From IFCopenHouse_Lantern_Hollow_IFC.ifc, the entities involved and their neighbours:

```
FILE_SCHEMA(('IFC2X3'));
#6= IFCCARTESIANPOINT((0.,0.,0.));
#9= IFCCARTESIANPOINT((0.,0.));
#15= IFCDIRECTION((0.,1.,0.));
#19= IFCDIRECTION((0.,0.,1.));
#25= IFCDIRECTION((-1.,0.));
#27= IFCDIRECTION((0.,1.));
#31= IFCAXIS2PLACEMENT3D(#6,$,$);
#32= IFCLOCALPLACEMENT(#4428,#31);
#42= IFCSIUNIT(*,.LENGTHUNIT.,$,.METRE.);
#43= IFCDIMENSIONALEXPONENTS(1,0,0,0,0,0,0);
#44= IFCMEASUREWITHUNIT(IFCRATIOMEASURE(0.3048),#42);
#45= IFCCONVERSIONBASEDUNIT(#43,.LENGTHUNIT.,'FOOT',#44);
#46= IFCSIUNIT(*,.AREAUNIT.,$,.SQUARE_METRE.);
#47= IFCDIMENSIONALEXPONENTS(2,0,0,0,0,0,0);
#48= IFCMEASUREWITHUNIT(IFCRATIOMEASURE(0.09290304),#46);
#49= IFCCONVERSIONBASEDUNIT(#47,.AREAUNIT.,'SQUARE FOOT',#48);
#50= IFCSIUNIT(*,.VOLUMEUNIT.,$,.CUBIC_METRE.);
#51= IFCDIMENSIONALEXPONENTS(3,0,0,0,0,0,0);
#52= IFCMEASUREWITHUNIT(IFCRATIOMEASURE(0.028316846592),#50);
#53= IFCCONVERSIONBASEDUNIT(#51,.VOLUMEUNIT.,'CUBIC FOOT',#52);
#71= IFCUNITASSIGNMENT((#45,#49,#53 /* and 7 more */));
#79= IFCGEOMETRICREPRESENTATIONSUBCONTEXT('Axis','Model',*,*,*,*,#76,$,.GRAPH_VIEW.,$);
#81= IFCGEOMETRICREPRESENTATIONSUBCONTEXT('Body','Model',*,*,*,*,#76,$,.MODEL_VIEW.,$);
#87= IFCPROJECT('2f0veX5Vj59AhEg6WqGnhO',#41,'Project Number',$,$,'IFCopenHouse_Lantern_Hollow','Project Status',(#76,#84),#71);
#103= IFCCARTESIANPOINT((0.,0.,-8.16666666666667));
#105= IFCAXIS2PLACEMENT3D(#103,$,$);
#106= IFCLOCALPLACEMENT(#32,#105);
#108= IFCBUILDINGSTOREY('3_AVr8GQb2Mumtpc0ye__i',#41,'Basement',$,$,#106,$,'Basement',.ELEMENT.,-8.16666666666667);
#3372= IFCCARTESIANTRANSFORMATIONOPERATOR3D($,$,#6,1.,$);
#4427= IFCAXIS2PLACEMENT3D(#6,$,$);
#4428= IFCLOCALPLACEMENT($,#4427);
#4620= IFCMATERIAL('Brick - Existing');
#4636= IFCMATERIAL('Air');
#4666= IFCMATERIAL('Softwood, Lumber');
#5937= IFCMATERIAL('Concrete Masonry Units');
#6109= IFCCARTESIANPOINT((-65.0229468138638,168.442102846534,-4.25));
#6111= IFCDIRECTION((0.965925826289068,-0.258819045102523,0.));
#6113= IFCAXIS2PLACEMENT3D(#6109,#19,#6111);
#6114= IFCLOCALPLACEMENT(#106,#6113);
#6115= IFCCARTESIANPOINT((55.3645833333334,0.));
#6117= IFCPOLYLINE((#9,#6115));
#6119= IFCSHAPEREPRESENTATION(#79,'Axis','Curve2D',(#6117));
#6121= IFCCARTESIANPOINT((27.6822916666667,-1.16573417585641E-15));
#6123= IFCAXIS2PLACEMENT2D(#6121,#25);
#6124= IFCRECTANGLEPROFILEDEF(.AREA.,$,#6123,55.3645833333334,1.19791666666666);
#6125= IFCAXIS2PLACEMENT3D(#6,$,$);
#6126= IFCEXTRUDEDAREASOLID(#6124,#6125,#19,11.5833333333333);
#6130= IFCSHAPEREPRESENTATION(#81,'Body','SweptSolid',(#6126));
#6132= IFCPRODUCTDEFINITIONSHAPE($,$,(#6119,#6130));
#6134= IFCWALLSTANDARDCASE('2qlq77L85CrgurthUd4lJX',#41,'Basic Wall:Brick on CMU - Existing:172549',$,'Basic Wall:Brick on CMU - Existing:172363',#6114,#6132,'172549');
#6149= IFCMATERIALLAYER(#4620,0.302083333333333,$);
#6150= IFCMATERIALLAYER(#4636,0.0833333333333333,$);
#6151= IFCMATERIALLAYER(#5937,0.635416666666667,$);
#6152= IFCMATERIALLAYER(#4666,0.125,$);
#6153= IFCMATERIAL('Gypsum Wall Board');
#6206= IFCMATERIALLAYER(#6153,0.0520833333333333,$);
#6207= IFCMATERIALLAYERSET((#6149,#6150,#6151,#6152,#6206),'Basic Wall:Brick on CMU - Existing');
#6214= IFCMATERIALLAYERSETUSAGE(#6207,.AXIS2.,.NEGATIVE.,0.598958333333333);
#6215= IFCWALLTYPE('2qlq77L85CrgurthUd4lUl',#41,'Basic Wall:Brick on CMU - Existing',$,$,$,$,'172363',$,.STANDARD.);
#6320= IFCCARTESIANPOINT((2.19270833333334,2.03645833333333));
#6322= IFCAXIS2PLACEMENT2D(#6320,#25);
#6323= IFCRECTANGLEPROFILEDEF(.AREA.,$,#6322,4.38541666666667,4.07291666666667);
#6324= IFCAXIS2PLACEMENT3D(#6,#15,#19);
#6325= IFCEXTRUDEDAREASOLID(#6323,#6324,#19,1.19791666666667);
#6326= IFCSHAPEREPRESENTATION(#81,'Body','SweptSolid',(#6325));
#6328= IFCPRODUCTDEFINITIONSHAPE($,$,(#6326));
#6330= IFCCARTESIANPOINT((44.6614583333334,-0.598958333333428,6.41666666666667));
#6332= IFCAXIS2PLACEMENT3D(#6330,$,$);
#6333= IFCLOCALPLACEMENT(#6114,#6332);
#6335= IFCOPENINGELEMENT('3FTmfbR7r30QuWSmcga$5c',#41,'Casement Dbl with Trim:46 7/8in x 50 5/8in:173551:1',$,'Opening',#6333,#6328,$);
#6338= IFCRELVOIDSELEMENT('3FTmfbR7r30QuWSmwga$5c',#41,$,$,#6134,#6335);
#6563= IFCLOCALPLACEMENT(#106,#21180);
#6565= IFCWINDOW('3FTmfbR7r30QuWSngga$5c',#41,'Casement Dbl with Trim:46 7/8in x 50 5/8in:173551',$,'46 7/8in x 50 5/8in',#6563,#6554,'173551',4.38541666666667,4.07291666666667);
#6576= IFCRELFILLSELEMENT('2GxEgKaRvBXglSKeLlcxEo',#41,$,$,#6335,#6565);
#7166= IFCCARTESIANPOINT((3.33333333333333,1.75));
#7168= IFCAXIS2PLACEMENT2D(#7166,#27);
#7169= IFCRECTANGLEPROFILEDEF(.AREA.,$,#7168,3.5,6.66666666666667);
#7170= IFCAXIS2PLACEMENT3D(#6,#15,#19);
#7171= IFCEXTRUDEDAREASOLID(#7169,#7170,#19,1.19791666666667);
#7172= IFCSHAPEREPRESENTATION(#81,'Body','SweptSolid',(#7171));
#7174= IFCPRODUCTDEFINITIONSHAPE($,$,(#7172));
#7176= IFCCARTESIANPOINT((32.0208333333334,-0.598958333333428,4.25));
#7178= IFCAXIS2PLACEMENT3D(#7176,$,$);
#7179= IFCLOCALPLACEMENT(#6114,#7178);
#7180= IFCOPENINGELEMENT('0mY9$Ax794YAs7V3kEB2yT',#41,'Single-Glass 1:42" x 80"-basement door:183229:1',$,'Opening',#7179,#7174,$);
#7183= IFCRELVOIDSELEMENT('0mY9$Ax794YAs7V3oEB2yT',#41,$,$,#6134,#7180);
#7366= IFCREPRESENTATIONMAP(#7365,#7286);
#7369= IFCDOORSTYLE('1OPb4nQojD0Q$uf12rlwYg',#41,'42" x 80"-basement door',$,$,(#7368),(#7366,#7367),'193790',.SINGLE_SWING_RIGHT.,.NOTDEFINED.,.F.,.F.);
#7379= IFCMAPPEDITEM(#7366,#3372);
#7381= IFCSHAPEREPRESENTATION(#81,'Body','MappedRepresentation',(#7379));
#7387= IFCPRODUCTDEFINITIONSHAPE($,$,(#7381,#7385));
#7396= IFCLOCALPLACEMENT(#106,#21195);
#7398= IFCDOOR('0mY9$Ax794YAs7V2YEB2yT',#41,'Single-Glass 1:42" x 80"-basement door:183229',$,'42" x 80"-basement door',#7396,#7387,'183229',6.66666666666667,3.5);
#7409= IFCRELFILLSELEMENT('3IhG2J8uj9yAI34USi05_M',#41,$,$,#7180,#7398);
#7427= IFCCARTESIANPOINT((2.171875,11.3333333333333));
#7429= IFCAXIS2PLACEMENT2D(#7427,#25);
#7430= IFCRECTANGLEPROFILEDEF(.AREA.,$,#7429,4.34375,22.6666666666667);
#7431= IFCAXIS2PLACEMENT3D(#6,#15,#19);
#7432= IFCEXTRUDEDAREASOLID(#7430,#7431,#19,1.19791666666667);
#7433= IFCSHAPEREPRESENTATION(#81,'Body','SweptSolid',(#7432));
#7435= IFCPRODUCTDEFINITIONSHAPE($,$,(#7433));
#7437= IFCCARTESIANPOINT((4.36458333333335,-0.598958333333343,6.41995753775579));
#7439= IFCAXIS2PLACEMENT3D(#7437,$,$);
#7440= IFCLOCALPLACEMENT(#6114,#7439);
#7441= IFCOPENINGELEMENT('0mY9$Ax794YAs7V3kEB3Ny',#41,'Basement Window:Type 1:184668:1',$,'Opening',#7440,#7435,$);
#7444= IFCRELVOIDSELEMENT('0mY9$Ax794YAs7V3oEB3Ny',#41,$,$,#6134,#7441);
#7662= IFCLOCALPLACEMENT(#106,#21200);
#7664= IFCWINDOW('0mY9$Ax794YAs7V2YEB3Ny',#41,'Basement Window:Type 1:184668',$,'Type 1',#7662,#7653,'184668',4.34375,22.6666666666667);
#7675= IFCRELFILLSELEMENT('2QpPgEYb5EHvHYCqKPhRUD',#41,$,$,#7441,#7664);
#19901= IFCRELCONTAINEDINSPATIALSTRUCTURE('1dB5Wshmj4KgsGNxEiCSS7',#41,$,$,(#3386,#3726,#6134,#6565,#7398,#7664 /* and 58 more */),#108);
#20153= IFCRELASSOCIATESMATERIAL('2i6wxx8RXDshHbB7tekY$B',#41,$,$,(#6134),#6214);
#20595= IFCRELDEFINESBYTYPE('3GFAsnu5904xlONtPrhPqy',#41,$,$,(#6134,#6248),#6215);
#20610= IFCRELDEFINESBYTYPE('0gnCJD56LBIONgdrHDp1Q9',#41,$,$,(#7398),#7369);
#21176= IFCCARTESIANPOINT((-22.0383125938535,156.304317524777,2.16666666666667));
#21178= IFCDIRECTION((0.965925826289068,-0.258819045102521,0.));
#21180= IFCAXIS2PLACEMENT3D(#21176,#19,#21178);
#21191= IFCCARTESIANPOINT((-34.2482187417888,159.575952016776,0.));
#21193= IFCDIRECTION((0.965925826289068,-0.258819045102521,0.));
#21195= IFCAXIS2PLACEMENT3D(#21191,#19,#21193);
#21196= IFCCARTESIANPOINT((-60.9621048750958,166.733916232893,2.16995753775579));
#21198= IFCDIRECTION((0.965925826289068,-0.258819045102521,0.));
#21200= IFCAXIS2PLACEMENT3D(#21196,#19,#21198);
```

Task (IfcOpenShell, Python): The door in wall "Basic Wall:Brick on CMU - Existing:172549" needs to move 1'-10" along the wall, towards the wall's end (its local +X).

```python
import ifcopenshell
import ifcopenshell.api.geometry
import ifcopenshell.util.placement
import ifcopenshell.util.unit

model = ifcopenshell.open("IFCopenHouse_Lantern_Hollow_IFC.ifc")
unit_scale = ifcopenshell.util.unit.calculate_unit_scale(model)

door = model.by_guid("0mY9$Ax794YAs7V2YEB2yT")
opening = door.FillsVoids[0].RelatingOpeningElement
wall = opening.VoidsElements[0].RelatingBuildingElement

wall_matrix = ifcopenshell.util.placement.get_local_placement(wall.ObjectPlacement)
shift = wall_matrix[:3, 0] * 22 * 0.0254 / unit_scale
before = ifcopenshell.util.placement.get_local_placement(door.ObjectPlacement)[:3, 3].copy()

# The door is not placed relative to its opening, so move both.
for product in (opening, door):
    matrix = ifcopenshell.util.placement.get_local_placement(product.ObjectPlacement)
    matrix[:3, 3] += shift
    ifcopenshell.api.geometry.edit_object_placement(model, product=product, matrix=matrix, is_si=False)

after = ifcopenshell.util.placement.get_local_placement(door.ObjectPlacement)[:3, 3]
print("door moved by", (after - before).round(3) + 0.0)

model.write("IFCopenHouse_Lantern_Hollow_IFC-out.ifc")
```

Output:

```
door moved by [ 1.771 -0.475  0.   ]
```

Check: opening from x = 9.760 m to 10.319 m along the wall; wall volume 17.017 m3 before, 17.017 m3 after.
